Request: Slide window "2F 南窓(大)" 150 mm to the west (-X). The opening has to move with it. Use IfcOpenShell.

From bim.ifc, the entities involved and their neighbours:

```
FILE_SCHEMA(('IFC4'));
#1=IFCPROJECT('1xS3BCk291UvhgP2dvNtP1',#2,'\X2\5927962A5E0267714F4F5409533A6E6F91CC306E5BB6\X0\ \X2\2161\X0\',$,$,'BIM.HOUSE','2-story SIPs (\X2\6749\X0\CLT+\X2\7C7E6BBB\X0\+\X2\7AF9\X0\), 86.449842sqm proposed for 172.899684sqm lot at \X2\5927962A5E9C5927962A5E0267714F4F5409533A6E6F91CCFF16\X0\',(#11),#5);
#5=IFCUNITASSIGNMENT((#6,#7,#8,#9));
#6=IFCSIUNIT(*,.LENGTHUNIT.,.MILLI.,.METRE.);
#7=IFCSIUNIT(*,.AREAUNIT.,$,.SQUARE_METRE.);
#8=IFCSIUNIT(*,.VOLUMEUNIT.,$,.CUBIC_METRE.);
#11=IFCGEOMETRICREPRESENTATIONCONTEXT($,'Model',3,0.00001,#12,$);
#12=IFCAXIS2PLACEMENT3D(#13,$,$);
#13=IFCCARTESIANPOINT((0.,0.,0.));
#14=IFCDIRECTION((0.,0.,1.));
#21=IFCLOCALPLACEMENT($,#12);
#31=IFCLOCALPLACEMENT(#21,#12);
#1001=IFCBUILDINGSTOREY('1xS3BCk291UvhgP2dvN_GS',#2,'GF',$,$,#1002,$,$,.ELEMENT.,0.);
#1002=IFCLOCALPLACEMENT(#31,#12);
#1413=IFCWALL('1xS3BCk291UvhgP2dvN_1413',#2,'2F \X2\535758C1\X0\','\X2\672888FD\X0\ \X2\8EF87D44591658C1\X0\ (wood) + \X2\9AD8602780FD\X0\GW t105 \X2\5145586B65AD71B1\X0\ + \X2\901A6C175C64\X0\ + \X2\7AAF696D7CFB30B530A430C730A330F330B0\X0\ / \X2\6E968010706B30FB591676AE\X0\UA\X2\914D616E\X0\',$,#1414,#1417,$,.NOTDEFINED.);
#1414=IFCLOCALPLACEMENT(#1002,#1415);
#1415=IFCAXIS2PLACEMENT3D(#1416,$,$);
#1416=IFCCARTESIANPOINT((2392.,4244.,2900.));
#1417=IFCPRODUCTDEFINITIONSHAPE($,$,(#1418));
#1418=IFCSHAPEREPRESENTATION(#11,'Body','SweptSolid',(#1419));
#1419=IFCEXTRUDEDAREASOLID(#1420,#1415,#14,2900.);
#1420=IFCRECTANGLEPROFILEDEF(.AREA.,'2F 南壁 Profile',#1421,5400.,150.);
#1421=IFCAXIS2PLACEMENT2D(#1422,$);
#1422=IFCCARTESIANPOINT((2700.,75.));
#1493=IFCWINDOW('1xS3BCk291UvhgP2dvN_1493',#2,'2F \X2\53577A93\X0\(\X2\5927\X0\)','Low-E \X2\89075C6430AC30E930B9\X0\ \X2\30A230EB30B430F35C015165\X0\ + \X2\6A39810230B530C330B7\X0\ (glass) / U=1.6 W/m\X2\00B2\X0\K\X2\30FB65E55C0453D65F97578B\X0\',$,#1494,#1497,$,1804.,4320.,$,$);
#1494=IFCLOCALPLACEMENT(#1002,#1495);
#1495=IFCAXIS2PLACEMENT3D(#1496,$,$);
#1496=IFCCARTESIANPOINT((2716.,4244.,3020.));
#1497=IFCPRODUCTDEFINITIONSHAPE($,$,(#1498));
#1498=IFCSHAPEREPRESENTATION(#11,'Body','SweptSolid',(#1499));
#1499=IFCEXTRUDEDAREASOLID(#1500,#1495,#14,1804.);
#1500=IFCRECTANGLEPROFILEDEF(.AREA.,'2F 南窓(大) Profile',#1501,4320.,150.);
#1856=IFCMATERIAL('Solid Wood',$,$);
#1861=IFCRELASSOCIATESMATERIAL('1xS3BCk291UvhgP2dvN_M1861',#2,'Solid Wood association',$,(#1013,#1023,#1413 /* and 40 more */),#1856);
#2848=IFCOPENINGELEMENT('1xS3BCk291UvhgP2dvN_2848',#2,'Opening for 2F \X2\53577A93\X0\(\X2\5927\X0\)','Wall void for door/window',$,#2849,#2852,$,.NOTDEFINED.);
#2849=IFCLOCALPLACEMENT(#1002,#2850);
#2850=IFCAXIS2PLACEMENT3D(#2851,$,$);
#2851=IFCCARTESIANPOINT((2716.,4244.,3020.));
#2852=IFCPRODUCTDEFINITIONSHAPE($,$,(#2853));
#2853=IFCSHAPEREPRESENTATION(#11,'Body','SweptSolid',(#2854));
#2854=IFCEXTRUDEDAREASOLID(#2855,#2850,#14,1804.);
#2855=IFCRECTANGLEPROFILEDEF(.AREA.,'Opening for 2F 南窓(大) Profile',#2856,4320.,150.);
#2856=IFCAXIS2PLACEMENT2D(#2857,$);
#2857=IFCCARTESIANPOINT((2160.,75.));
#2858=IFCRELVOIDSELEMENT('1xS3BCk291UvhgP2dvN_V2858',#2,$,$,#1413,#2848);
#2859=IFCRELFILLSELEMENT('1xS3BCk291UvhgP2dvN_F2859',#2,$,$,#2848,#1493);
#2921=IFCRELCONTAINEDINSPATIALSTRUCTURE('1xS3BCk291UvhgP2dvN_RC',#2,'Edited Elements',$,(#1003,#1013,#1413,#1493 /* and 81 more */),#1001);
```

```python
import ifcopenshell
import ifcopenshell.api.geometry
import ifcopenshell.util.placement
import ifcopenshell.util.unit

model = ifcopenshell.open("bim.ifc")
unit_scale = ifcopenshell.util.unit.calculate_unit_scale(model)

window = model.by_id(1493)
opening = window.FillsVoids[0].RelatingOpeningElement
wall = opening.VoidsElements[0].RelatingBuildingElement

wall_matrix = ifcopenshell.util.placement.get_local_placement(wall.ObjectPlacement)
shift = wall_matrix[:3, 0] * -0.15 / unit_scale
before = ifcopenshell.util.placement.get_local_placement(window.ObjectPlacement)[:3, 3].copy()

# The window is not placed relative to its opening, so move both.
for product in (opening, window):
    matrix = ifcopenshell.util.placement.get_local_placement(product.ObjectPlacement)
    matrix[:3, 3] += shift
    ifcopenshell.api.geometry.edit_object_placement(model, product=product, matrix=matrix, is_si=False)

after = ifcopenshell.util.placement.get_local_placement(window.ObjectPlacement)[:3, 3]
print("window moved by", (after - before).round(3) + 0.0)

model.write("bim_rev.ifc")
```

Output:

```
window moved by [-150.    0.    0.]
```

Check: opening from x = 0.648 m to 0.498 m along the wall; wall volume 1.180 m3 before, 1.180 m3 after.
